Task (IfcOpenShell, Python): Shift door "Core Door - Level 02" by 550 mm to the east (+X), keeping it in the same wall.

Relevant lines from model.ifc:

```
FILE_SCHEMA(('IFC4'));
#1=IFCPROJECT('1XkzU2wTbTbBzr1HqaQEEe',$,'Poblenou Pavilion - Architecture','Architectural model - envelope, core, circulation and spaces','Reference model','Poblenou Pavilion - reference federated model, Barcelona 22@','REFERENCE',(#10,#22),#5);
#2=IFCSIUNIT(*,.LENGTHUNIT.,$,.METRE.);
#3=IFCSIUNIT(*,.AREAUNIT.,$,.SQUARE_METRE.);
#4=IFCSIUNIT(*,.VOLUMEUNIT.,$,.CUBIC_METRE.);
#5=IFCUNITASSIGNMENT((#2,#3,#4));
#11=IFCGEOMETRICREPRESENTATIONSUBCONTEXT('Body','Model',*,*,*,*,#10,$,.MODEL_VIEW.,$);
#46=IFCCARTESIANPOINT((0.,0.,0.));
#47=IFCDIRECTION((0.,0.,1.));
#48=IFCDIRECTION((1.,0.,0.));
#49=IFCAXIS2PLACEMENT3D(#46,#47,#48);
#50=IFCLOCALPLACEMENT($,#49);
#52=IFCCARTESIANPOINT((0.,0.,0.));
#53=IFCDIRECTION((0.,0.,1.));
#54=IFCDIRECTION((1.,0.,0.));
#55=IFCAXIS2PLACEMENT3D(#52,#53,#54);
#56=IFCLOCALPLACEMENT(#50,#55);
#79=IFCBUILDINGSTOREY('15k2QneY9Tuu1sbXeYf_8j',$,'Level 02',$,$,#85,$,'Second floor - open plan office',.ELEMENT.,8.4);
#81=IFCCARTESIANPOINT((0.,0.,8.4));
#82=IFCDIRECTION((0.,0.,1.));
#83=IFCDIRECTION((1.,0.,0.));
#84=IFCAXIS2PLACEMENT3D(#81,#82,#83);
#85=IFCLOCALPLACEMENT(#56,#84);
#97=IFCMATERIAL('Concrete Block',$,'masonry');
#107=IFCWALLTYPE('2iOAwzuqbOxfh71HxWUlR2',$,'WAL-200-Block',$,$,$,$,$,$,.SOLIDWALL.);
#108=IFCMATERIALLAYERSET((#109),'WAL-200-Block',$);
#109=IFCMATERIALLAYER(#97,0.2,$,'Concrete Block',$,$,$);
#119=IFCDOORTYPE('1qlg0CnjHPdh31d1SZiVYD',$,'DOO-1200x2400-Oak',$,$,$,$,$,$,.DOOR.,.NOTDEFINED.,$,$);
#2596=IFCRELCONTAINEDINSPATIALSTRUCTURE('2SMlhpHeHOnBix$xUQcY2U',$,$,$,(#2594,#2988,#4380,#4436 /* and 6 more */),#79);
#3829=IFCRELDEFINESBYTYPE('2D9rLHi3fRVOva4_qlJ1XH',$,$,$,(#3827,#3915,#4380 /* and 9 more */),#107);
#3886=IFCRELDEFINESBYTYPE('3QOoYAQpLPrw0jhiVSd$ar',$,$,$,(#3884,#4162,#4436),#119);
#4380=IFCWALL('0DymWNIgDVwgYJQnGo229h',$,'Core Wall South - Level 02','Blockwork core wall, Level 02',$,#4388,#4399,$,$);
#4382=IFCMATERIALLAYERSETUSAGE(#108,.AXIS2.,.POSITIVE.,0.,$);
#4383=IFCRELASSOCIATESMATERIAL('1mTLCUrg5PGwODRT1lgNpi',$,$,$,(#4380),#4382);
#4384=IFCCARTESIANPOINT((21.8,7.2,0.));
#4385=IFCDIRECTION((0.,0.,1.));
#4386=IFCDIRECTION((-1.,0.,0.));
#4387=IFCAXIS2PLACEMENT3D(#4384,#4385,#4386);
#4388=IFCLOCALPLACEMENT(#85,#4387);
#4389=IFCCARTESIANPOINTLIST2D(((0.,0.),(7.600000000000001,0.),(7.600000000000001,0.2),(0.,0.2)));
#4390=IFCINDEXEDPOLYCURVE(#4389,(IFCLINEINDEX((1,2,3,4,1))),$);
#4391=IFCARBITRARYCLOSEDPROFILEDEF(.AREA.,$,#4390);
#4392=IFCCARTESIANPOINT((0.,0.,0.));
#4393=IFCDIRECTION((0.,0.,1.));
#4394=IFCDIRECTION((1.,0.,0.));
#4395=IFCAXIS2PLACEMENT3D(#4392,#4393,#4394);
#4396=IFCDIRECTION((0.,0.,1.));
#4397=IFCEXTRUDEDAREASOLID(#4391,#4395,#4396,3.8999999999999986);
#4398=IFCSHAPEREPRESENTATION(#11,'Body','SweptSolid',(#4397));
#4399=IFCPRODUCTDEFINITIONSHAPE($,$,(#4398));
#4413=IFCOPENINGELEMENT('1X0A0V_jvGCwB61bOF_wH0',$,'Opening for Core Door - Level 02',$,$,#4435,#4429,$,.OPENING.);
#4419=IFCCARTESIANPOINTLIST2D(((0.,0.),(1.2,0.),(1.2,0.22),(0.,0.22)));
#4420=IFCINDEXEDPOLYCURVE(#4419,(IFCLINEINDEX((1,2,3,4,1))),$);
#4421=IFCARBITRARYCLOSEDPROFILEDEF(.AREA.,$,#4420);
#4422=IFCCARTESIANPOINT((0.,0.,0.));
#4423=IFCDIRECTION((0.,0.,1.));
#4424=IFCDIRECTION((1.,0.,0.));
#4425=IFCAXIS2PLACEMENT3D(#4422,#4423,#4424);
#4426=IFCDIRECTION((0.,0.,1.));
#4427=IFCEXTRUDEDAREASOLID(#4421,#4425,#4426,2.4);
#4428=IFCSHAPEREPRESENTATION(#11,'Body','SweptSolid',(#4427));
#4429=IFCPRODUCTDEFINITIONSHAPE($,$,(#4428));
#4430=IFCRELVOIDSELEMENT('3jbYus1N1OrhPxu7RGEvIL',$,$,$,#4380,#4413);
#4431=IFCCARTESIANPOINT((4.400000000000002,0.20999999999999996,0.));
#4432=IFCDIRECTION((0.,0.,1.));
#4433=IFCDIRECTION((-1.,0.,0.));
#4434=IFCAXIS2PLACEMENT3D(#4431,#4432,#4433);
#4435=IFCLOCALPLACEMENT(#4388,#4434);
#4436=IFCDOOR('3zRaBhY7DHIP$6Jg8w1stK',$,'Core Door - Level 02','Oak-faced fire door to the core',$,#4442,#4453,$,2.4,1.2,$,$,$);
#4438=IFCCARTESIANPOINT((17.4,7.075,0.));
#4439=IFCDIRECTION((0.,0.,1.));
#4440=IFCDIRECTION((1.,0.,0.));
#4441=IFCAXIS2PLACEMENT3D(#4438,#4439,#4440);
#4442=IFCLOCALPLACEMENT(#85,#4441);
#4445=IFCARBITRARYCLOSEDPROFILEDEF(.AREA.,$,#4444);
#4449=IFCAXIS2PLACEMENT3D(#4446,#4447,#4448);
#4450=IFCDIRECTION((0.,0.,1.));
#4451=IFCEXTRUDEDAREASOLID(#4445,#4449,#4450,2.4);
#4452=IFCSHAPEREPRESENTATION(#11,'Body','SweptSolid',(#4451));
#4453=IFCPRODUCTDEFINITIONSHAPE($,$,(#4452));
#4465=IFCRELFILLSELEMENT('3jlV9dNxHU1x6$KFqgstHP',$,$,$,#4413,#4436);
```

```python
import ifcopenshell
import ifcopenshell.api.geometry
import ifcopenshell.util.placement
import ifcopenshell.util.unit

model = ifcopenshell.open("model.ifc")
unit_scale = ifcopenshell.util.unit.calculate_unit_scale(model)

door = model.by_guid("3zRaBhY7DHIP$6Jg8w1stK")
opening = door.FillsVoids[0].RelatingOpeningElement
wall = opening.VoidsElements[0].RelatingBuildingElement

wall_matrix = ifcopenshell.util.placement.get_local_placement(wall.ObjectPlacement)
shift = wall_matrix[:3, 0] * -0.55 / unit_scale
before = ifcopenshell.util.placement.get_local_placement(door.ObjectPlacement)[:3, 3].copy()

# The door is not placed relative to its opening, so move both.
for product in (opening, door):
    matrix = ifcopenshell.util.placement.get_local_placement(product.ObjectPlacement)
    matrix[:3, 3] += shift
    ifcopenshell.api.geometry.edit_object_placement(model, product=product, matrix=matrix, is_si=False)

after = ifcopenshell.util.placement.get_local_placement(door.ObjectPlacement)[:3, 3]
print("door moved by", (after - before).round(3) + 0.0)

model.write("model-out.ifc")
```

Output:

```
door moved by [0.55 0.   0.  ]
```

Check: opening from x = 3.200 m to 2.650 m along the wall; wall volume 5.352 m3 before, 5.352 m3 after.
